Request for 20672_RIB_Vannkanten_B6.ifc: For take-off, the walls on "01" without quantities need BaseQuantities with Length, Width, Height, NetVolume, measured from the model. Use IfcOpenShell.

First a look at what the model holds.

```python
import ifcopenshell
import ifcopenshell.util.element
import ifcopenshell.util.unit

model = ifcopenshell.open("20672_RIB_Vannkanten_B6.ifc")
print(model.schema)
for unit_type in ("LENGTHUNIT", "AREAUNIT", "VOLUMEUNIT"):
    print(unit_type, ifcopenshell.util.unit.calculate_unit_scale(model, unit_type))
storey = next(s for s in model.by_type("IfcBuildingStorey") if s.Name == "01")
walls = [e for e in ifcopenshell.util.element.get_decomposition(storey) if e.is_a("IfcWall")]
for e in sorted(walls, key=lambda e: e.id()):
    print(e.id(), e.is_a(), e.Name, list(ifcopenshell.util.element.get_psets(e, qtos_only=True)), sep=" | ")
```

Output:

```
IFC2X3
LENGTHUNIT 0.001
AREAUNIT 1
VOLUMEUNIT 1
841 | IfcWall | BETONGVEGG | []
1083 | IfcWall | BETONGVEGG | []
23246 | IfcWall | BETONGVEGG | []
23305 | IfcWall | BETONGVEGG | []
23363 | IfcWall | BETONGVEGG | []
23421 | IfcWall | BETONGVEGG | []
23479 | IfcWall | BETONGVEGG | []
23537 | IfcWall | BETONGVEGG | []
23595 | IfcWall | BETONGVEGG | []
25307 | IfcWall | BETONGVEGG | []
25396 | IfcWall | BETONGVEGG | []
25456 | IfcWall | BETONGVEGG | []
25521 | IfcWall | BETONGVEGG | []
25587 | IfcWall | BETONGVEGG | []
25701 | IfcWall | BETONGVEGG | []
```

```python
import ifcopenshell
import ifcopenshell.api.pset
import ifcopenshell.geom
import ifcopenshell.util.element
import ifcopenshell.util.shape
import ifcopenshell.util.unit

model = ifcopenshell.open("20672_RIB_Vannkanten_B6.ifc")
unit_scale = ifcopenshell.util.unit.calculate_unit_scale(model)
volume_scale = ifcopenshell.util.unit.calculate_unit_scale(model, "VOLUMEUNIT")
settings = ifcopenshell.geom.settings()

storey = next(s for s in model.by_type("IfcBuildingStorey") if s.Name == "01")
walls = [e for e in ifcopenshell.util.element.get_decomposition(storey) if e.is_a("IfcWall")]

for e in sorted(walls, key=lambda e: e.id()):
    if ifcopenshell.util.element.get_psets(e, qtos_only=True, should_inherit=False):
        continue
    # Geometry comes back in metres, in the element's own axes.
    shape = ifcopenshell.geom.create_shape(settings, e)
    values = {
        "Length": ifcopenshell.util.shape.get_x(shape.geometry) / unit_scale,
        "Width": ifcopenshell.util.shape.get_y(shape.geometry) / unit_scale,
        "Height": ifcopenshell.util.shape.get_z(shape.geometry) / unit_scale,
        "NetVolume": ifcopenshell.util.shape.get_volume(shape.geometry) / volume_scale,
    }
    qto = ifcopenshell.api.pset.add_qto(model, product=e, name="BaseQuantities")
    ifcopenshell.api.pset.edit_qto(model, qto=qto, properties=values)
    print(e.id(), {k: round(v, 3) for k, v in values.items()})

model.write("20672_RIB_Vannkanten_B6_edited.ifc")
```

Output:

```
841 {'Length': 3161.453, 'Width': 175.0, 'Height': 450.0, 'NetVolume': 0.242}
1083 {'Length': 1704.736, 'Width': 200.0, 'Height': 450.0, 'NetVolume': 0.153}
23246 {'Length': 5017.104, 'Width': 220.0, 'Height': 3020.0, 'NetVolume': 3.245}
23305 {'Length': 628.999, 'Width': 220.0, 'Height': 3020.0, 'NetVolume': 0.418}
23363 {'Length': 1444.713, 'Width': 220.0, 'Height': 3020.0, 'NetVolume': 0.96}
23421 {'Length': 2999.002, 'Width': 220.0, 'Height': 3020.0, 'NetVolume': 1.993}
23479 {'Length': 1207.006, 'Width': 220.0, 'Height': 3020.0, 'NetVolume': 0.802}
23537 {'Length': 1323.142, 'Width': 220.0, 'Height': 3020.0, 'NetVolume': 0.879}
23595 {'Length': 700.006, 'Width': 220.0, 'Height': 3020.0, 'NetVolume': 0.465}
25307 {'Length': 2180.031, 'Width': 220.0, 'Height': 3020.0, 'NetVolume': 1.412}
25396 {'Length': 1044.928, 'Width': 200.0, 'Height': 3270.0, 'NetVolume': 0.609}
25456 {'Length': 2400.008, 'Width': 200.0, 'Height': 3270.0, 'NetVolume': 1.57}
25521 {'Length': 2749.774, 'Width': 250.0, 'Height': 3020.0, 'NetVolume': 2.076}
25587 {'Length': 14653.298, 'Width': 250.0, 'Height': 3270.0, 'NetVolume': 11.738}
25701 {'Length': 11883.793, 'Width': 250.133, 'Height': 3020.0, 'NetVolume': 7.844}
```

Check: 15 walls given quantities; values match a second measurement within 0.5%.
